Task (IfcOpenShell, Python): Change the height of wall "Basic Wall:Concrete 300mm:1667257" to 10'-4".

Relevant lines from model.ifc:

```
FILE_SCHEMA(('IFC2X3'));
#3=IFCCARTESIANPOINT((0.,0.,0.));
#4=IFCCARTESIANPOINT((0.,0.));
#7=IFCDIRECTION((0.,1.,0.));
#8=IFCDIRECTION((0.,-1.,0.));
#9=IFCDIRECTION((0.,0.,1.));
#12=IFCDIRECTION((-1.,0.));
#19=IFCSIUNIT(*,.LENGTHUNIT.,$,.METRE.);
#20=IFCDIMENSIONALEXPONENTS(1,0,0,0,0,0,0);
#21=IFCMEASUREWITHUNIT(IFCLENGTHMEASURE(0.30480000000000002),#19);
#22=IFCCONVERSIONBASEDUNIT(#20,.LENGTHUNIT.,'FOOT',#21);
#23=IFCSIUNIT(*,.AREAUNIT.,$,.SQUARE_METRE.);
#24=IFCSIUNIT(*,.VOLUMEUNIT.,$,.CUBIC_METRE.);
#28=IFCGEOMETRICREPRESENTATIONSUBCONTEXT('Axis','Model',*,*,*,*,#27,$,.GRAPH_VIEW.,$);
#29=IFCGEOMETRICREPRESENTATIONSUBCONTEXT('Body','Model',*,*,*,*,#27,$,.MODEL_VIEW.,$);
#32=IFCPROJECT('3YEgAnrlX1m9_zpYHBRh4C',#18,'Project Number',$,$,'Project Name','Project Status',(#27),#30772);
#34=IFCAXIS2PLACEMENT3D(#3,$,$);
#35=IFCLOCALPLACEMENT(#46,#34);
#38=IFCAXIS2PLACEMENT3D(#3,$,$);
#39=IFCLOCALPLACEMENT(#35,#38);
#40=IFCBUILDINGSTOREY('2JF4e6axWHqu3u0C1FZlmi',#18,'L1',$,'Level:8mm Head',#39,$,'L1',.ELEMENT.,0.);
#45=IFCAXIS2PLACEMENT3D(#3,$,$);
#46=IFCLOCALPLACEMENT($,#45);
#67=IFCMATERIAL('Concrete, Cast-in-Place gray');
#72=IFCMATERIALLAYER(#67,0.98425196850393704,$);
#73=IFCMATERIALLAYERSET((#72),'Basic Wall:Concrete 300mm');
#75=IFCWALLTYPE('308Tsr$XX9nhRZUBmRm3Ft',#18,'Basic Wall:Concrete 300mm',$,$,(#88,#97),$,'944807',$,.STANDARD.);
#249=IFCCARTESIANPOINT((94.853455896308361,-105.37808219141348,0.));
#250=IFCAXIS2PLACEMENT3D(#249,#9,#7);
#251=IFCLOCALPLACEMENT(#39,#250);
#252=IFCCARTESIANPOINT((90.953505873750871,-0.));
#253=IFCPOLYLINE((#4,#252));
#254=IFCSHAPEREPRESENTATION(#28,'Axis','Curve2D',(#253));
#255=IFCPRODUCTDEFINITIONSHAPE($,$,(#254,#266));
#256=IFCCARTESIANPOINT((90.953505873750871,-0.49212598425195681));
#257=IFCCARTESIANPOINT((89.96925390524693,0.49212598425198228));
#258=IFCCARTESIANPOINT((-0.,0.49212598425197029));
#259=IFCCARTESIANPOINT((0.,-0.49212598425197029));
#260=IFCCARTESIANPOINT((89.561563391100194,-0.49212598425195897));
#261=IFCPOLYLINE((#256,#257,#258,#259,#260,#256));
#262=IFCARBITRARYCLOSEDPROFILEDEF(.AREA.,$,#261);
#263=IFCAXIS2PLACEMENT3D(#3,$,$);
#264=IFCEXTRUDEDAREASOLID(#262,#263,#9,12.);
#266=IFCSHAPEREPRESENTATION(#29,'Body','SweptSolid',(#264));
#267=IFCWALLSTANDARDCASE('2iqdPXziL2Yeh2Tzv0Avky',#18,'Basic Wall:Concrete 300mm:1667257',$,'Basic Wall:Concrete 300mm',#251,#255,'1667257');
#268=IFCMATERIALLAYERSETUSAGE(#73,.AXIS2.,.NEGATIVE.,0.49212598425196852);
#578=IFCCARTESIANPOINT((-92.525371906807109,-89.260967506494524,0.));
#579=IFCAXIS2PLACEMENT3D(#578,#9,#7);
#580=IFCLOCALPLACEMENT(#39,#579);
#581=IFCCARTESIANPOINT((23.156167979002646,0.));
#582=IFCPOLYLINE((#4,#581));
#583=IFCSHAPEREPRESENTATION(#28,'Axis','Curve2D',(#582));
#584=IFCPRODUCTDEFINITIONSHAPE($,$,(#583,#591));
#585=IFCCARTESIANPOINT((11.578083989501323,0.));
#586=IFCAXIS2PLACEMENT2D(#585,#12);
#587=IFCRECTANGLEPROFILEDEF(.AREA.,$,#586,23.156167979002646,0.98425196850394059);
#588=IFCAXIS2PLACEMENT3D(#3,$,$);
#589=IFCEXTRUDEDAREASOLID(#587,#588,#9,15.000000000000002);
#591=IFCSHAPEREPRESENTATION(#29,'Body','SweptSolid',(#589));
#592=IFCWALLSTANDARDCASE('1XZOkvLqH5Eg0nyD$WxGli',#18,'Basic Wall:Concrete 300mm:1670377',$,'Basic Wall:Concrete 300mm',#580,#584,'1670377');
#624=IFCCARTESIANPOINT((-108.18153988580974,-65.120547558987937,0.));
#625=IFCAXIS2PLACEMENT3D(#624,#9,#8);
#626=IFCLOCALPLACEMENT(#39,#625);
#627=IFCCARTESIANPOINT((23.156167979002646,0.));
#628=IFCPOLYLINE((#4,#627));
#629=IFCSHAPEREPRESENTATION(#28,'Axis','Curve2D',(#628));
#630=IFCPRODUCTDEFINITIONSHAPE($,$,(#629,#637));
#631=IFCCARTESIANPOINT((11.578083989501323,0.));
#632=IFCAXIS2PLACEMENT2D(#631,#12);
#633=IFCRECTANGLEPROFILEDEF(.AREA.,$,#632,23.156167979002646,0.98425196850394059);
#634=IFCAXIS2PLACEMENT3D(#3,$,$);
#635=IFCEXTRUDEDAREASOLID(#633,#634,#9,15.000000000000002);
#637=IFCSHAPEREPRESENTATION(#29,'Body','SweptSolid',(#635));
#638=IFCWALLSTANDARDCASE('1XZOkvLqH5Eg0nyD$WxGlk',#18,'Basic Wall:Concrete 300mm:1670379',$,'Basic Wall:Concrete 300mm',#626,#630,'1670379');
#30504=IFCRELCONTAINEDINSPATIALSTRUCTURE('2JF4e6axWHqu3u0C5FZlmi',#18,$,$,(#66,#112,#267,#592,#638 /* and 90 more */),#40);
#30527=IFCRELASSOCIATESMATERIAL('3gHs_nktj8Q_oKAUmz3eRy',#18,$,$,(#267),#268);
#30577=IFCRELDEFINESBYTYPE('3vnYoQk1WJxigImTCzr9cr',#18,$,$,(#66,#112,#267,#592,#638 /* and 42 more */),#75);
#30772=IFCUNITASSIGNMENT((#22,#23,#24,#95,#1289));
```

```python
import ifcopenshell
import ifcopenshell.geom
import ifcopenshell.util.representation
import ifcopenshell.util.shape
import ifcopenshell.util.unit

model = ifcopenshell.open("model.ifc")
unit_scale = ifcopenshell.util.unit.calculate_unit_scale(model)
settings = ifcopenshell.geom.settings()


def volume(element):
    """Net volume in cubic metres, openings subtracted."""
    shape = ifcopenshell.geom.create_shape(settings, element)
    return ifcopenshell.util.shape.get_volume(shape.geometry)


wall = model.by_guid("2iqdPXziL2Yeh2Tzv0Avky")
before = volume(wall)

body = ifcopenshell.util.representation.get_representation(wall, "Model", "Body")
solid = body.Items[0]
old_height = solid.Depth
solid.Depth = 124 * 0.0254 / unit_scale
after = volume(wall)

print(f"height {old_height:g} -> {solid.Depth:g}, volume {before:.3f} -> {after:.3f} m3")

model.write("model_v2.ifc")
```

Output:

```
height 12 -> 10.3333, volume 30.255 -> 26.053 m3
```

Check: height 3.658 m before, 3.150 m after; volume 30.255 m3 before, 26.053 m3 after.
